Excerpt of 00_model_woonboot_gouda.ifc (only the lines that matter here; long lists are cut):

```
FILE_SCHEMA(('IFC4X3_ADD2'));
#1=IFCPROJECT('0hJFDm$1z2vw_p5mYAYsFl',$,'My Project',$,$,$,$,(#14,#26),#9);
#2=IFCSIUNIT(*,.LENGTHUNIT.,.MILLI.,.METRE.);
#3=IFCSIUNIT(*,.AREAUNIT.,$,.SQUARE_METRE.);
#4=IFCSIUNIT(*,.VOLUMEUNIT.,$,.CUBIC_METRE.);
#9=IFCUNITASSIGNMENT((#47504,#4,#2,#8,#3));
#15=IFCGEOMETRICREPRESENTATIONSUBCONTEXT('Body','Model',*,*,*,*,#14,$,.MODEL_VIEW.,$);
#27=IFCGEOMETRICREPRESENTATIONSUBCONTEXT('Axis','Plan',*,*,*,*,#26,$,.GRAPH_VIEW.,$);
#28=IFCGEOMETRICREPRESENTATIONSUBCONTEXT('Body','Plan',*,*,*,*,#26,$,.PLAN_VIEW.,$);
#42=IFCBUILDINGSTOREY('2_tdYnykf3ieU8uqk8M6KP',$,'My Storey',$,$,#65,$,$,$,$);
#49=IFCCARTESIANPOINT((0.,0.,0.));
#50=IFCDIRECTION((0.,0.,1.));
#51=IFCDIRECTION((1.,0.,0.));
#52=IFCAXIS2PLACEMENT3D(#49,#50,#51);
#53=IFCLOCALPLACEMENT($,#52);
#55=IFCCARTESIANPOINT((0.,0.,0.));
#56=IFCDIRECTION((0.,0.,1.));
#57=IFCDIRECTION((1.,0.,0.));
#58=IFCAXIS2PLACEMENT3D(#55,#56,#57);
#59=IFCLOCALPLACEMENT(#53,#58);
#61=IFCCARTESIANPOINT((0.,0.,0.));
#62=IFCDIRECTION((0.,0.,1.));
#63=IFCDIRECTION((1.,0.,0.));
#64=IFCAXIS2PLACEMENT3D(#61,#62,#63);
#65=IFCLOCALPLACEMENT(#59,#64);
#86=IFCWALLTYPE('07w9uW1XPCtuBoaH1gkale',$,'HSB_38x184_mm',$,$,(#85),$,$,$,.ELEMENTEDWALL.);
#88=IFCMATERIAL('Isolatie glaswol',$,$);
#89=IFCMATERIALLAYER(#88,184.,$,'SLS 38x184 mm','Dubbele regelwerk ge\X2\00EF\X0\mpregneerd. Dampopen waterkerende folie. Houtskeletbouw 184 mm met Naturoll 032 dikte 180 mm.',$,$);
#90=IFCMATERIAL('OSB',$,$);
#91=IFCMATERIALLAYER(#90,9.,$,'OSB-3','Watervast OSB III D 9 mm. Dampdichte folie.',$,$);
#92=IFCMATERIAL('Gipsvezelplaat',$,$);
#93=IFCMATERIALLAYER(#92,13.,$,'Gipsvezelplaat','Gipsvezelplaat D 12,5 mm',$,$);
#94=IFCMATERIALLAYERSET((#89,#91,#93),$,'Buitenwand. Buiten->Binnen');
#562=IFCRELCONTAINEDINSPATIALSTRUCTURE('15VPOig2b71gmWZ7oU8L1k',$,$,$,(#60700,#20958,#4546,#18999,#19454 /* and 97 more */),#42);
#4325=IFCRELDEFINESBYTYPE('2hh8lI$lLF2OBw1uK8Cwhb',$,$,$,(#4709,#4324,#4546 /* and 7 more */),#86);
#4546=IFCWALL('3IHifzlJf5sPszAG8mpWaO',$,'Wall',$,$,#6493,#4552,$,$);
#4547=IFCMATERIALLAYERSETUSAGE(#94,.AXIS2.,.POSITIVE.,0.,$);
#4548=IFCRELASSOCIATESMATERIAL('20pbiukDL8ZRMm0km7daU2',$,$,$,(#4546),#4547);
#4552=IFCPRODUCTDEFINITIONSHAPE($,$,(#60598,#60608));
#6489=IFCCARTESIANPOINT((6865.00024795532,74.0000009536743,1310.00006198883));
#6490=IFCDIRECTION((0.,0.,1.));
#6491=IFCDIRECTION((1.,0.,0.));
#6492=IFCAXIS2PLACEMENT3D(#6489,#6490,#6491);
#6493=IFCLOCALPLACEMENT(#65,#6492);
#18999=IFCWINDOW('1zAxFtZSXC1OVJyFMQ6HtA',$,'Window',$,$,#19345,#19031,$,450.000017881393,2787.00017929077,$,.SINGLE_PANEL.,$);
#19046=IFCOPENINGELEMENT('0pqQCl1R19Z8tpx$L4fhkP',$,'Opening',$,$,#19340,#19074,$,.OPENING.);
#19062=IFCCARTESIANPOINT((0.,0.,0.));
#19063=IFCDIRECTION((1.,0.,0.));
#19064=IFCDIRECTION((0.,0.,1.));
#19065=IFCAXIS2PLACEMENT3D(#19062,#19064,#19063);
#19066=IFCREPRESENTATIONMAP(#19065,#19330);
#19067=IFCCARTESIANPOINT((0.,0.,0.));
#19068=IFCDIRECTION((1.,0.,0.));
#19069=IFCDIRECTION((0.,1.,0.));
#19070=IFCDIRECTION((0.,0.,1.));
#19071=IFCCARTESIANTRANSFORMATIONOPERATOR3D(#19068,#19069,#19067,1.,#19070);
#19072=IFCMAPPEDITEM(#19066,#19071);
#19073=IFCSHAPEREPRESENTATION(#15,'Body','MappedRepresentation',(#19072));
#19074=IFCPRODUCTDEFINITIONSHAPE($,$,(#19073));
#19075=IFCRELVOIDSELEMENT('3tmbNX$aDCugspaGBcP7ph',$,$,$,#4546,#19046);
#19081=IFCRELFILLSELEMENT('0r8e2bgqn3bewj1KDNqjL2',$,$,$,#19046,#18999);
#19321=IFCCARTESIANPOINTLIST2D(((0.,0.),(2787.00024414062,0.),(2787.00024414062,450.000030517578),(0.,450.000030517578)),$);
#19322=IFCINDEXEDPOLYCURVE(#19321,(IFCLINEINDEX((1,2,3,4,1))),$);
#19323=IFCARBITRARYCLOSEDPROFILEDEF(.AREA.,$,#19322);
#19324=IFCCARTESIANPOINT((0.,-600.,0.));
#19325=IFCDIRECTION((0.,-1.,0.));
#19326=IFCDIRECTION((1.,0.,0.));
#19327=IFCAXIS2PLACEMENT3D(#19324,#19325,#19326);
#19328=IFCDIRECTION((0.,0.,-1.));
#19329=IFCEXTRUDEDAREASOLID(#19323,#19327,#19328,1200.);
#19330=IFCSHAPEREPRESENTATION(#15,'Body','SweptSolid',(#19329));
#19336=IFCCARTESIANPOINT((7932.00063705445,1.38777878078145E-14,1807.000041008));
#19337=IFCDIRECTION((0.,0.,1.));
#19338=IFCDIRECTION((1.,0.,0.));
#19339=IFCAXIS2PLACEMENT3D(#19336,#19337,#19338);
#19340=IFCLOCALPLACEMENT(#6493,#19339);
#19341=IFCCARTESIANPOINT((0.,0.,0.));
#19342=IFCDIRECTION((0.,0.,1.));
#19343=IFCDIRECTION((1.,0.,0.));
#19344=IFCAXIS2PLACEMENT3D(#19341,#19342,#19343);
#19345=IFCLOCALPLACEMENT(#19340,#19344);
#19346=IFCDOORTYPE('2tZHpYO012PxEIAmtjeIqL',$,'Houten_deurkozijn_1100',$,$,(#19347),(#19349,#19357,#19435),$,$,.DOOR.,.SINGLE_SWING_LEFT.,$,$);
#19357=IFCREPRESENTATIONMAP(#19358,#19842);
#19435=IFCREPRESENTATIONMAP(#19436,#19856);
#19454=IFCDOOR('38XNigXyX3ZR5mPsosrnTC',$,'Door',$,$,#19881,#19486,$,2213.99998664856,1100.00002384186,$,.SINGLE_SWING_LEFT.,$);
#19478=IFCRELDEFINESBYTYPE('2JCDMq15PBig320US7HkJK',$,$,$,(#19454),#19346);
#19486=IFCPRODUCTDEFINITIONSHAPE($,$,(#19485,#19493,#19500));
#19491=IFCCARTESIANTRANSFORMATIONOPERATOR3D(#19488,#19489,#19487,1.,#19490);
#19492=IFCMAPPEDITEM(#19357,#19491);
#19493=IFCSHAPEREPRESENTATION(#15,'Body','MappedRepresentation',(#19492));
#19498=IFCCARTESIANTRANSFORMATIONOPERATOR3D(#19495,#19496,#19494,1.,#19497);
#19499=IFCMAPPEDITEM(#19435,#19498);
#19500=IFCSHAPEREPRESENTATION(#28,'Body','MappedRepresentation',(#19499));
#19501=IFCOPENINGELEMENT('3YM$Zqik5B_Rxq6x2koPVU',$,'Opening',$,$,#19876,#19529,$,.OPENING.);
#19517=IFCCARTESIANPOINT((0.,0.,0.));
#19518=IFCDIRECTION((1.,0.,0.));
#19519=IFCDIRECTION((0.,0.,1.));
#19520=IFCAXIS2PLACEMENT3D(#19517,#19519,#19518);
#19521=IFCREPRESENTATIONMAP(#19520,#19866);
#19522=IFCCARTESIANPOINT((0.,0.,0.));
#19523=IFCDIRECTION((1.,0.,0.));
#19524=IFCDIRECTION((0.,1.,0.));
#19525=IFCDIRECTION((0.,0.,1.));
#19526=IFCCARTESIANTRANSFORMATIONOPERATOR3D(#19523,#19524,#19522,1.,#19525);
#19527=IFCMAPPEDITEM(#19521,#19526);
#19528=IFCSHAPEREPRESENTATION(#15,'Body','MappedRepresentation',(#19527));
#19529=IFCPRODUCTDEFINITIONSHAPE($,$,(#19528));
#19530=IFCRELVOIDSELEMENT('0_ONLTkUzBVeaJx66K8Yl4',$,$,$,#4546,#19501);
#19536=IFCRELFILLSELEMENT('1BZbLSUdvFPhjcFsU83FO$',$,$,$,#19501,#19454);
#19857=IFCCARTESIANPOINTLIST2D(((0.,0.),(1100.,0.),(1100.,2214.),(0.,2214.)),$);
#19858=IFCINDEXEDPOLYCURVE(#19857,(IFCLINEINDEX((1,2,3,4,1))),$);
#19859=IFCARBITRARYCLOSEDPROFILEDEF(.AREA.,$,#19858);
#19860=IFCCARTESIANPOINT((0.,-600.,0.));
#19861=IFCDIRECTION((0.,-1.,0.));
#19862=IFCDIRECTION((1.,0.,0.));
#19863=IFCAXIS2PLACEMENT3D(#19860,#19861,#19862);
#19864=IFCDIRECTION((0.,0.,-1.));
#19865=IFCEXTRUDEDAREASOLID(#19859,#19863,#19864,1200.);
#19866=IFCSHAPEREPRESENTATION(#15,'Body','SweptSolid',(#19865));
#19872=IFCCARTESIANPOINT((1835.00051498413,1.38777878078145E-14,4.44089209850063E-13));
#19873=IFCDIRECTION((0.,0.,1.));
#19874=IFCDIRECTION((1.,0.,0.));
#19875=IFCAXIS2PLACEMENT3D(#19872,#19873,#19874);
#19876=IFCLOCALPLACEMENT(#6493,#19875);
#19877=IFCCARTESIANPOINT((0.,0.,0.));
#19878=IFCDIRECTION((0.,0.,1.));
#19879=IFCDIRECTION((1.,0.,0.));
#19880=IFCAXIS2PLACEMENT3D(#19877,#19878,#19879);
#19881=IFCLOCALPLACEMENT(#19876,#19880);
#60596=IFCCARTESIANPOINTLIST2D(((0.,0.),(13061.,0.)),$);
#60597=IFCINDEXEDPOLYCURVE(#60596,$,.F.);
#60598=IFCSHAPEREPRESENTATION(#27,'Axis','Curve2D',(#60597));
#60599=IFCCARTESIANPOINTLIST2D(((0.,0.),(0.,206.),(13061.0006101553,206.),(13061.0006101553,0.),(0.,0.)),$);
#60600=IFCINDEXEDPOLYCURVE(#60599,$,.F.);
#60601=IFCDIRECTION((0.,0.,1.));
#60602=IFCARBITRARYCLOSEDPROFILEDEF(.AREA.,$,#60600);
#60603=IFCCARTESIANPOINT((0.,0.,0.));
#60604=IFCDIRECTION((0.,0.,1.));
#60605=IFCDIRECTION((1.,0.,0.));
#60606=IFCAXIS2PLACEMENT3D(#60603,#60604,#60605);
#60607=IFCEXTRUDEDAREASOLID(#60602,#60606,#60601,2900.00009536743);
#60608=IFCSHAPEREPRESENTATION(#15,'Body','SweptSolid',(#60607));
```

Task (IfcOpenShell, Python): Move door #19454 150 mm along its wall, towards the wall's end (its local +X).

```python
import ifcopenshell
import ifcopenshell.api.geometry
import ifcopenshell.util.placement
import ifcopenshell.util.unit

model = ifcopenshell.open("00_model_woonboot_gouda.ifc")
unit_scale = ifcopenshell.util.unit.calculate_unit_scale(model)

door = model.by_id(19454)
opening = door.FillsVoids[0].RelatingOpeningElement
wall = opening.VoidsElements[0].RelatingBuildingElement

wall_matrix = ifcopenshell.util.placement.get_local_placement(wall.ObjectPlacement)
shift = wall_matrix[:3, 0] * 0.15 / unit_scale
before = ifcopenshell.util.placement.get_local_placement(door.ObjectPlacement)[:3, 3].copy()

# The door is placed relative to its opening, so it follows when the opening moves.
matrix = ifcopenshell.util.placement.get_local_placement(opening.ObjectPlacement)
matrix[:3, 3] += shift
ifcopenshell.api.geometry.edit_object_placement(
    model, product=opening, matrix=matrix, is_si=False, should_transform_children=True
)

after = ifcopenshell.util.placement.get_local_placement(door.ObjectPlacement)[:3, 3]
print("door moved by", (after - before).round(3) + 0.0)

model.write("00_model_woonboot_gouda-out.ifc")
```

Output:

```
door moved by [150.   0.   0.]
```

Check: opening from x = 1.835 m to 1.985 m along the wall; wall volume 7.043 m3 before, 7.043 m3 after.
